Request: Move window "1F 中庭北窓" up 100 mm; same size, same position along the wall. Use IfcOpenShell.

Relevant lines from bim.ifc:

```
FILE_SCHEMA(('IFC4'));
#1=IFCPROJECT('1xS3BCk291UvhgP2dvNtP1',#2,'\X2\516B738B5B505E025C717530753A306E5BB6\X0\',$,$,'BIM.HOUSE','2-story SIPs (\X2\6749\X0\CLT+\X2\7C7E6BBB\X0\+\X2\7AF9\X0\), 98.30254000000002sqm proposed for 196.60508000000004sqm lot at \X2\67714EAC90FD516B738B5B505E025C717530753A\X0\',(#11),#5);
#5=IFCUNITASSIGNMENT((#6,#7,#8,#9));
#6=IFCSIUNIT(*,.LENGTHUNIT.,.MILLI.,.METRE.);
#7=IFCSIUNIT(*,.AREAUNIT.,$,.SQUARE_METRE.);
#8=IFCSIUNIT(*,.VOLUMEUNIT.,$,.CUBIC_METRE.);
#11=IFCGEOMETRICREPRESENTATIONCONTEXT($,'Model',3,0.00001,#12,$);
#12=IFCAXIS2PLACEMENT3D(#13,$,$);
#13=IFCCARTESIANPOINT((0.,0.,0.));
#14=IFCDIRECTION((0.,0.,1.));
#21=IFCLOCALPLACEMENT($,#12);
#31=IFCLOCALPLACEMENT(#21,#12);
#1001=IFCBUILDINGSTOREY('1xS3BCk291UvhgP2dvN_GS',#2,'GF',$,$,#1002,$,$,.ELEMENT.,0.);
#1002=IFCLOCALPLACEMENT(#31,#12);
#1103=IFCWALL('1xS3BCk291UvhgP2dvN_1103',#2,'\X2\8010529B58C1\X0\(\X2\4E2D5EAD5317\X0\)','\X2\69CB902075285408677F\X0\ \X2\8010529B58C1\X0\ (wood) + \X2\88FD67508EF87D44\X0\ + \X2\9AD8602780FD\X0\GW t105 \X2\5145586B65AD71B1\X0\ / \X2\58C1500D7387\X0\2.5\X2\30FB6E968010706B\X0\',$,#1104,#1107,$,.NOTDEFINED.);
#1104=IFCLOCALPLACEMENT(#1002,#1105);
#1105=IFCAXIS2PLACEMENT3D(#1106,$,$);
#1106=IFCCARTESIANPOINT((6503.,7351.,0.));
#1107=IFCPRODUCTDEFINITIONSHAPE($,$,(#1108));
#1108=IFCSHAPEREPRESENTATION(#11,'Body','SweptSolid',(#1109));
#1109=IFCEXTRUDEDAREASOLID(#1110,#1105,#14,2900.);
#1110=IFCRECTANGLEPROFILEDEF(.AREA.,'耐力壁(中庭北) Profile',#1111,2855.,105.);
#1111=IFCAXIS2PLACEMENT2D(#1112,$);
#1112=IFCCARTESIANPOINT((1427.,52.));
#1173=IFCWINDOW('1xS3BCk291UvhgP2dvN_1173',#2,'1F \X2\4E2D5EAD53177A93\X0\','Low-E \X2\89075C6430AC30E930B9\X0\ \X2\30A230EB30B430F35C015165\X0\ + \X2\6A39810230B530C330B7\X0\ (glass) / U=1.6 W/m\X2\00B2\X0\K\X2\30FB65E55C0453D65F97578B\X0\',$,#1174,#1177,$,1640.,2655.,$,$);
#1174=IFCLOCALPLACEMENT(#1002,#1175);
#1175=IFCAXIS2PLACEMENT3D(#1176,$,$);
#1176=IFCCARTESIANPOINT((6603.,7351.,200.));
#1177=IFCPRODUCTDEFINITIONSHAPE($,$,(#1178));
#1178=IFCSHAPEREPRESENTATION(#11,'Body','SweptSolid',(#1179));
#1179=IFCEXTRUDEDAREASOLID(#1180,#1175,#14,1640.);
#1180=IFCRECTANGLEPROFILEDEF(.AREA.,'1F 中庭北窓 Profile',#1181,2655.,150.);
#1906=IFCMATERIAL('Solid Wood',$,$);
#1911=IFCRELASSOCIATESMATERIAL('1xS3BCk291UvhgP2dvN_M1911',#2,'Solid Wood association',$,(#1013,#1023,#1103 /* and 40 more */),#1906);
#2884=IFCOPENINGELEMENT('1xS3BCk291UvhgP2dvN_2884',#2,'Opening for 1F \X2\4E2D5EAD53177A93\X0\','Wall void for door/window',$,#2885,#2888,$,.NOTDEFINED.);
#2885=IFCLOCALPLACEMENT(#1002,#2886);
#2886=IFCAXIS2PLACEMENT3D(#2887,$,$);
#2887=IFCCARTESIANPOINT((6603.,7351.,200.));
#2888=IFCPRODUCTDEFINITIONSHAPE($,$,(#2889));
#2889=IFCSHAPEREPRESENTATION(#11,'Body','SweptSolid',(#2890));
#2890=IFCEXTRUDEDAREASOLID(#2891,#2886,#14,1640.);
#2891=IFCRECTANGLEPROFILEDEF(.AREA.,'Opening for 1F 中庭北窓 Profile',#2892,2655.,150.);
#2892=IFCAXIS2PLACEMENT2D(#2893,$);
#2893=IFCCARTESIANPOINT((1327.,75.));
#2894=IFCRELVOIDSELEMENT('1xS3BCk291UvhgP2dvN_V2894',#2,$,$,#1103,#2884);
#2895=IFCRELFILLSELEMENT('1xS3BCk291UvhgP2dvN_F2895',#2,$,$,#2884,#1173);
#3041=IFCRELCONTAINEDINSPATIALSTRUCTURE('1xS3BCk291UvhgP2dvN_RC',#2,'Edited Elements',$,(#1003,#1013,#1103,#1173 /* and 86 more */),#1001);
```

```python
import numpy as np
import ifcopenshell
import ifcopenshell.api.geometry
import ifcopenshell.util.placement
import ifcopenshell.util.unit

model = ifcopenshell.open("bim.ifc")
unit_scale = ifcopenshell.util.unit.calculate_unit_scale(model)

window = model.by_guid("1xS3BCk291UvhgP2dvN_1173")
opening = window.FillsVoids[0].RelatingOpeningElement
dz = 0.1 / unit_scale

shift = np.array([0.0, 0.0, dz])
# The window is not placed relative to its opening, so move both.
for product in (opening, window):
    matrix = ifcopenshell.util.placement.get_local_placement(product.ObjectPlacement)
    matrix[:3, 3] += shift
    ifcopenshell.api.geometry.edit_object_placement(model, product=product, matrix=matrix, is_si=False)

print(f"moved by {dz * unit_scale:+.3f} m")

model.write("bim_edited.ifc")
```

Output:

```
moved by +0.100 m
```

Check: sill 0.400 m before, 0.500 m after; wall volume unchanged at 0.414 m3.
